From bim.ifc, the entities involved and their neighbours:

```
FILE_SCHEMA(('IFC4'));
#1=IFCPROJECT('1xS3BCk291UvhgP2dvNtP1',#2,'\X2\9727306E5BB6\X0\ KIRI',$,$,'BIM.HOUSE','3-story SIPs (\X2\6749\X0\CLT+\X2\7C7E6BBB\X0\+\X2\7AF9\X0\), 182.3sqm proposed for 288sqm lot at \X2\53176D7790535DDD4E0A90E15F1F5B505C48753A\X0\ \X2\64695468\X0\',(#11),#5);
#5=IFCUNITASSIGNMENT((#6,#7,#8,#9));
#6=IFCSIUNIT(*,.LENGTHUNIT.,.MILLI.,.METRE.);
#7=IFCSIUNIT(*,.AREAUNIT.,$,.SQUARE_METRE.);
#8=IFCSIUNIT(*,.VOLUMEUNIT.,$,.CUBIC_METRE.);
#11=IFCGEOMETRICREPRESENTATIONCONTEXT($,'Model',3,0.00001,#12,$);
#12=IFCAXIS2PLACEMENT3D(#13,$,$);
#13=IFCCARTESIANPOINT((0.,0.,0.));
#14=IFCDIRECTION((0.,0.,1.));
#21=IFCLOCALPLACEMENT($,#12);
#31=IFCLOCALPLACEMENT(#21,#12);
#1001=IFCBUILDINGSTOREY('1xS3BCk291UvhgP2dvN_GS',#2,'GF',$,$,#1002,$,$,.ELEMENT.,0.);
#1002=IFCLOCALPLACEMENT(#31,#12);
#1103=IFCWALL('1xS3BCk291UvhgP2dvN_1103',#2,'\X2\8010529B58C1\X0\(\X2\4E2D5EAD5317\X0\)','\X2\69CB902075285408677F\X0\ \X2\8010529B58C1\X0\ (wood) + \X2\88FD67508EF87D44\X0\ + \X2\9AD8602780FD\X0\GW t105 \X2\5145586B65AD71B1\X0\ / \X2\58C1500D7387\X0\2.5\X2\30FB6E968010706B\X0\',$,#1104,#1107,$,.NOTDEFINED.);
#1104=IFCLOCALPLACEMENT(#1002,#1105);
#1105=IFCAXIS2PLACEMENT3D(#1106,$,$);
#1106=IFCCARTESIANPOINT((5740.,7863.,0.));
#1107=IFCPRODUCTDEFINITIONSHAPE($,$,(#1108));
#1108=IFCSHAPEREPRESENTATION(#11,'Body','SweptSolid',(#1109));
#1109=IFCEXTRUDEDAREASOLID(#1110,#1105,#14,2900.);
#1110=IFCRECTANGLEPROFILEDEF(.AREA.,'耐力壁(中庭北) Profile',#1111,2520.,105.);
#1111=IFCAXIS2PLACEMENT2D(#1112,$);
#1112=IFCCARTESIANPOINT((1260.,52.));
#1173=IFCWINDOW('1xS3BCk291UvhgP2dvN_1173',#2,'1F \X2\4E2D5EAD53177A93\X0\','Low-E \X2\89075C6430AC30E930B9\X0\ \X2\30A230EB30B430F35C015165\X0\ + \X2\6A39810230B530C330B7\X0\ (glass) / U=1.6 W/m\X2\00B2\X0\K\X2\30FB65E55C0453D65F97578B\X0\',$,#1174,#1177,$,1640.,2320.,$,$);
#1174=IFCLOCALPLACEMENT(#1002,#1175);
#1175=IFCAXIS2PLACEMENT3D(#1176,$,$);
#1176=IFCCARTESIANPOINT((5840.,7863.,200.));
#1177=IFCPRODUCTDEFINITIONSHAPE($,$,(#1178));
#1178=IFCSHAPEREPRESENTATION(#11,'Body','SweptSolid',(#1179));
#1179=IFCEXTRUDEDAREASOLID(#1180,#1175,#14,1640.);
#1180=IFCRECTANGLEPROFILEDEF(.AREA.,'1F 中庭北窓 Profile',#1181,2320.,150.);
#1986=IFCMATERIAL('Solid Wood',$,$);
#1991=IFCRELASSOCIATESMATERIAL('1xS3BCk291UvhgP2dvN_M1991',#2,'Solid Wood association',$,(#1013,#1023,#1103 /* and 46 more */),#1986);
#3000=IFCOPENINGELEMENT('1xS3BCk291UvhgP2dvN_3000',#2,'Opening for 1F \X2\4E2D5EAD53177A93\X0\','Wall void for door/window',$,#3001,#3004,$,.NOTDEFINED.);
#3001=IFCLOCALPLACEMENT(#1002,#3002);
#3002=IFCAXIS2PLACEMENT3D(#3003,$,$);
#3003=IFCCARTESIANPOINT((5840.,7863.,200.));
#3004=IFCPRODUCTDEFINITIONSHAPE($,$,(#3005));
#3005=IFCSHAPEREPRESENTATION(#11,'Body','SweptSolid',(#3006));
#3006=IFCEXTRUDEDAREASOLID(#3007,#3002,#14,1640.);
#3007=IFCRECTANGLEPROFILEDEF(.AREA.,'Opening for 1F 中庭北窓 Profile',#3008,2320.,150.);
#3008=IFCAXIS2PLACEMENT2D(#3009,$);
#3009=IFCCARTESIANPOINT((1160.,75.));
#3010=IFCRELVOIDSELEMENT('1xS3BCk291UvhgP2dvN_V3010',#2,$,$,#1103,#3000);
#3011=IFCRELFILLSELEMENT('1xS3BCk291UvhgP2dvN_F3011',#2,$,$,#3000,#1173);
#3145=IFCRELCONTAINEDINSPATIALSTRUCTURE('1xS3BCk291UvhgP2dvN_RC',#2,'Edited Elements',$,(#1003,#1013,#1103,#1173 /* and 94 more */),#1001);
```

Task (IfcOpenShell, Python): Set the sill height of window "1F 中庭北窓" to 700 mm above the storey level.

```python
import numpy as np
import ifcopenshell
import ifcopenshell.api.geometry
import ifcopenshell.geom
import ifcopenshell.util.element
import ifcopenshell.util.placement
import ifcopenshell.util.shape
import ifcopenshell.util.unit

model = ifcopenshell.open("bim.ifc")
unit_scale = ifcopenshell.util.unit.calculate_unit_scale(model)

window = model.by_guid("1xS3BCk291UvhgP2dvN_1173")
opening = window.FillsVoids[0].RelatingOpeningElement
storey = ifcopenshell.util.element.get_container(window, ifc_class="IfcBuildingStorey")
level = ifcopenshell.util.placement.get_local_placement(storey.ObjectPlacement)[2, 3]

# The opening's origin need not be at the sill, so measure its lowest point.
shape = ifcopenshell.geom.create_shape(ifcopenshell.geom.settings(), opening)
bottom = ifcopenshell.util.shape.get_shape_bottom_elevation(shape, shape.geometry) / unit_scale
dz = level + 700.0 - bottom

shift = np.array([0.0, 0.0, dz])
# The window is not placed relative to its opening, so move both.
for product in (opening, window):
    matrix = ifcopenshell.util.placement.get_local_placement(product.ObjectPlacement)
    matrix[:3, 3] += shift
    ifcopenshell.api.geometry.edit_object_placement(model, product=product, matrix=matrix, is_si=False)

print(f"moved by {dz * unit_scale:+.3f} m")

model.write("bim_rev.ifc")
```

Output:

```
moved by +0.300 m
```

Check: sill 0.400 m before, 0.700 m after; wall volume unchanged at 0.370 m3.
